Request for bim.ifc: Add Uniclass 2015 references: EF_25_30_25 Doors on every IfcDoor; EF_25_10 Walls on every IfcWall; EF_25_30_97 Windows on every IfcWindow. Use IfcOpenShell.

First a look at what the model holds.

```python
import ifcopenshell

model = ifcopenshell.open("bim.ifc")
print(model.schema)
print("classifications:", [c.Name for c in model.by_type("IfcClassification")])
for ifc_class in ("IfcDoor", "IfcRoof", "IfcStair", "IfcWall", "IfcWindow"):
    print(ifc_class, len(model.by_type(ifc_class)))
```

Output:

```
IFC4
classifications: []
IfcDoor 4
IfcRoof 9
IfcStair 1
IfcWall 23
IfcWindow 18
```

```python
import ifcopenshell
import ifcopenshell.api.classification

model = ifcopenshell.open("bim.ifc")

system = ifcopenshell.api.classification.add_classification(model, classification="Uniclass 2015")

codes = {
    "IfcDoor": ("EF_25_30_25", "Doors"),
    "IfcWall": ("EF_25_10", "Walls"),
    "IfcWindow": ("EF_25_30_97", "Windows"),
}
for ifc_class, (code, name) in codes.items():
    products = model.by_type(ifc_class)
    ifcopenshell.api.classification.add_reference(
        model, products=products, classification=system, identification=code, name=name
    )
    print(code, len(products))

model.write("bim-out.ifc")
```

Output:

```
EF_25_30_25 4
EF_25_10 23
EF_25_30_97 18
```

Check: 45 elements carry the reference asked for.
